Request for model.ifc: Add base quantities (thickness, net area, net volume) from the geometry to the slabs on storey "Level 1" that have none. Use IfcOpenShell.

First a look at what the model holds.

```python
import ifcopenshell
import ifcopenshell.util.element
import ifcopenshell.util.unit

model = ifcopenshell.open("model.ifc")
print(model.schema)
for unit_type in ("LENGTHUNIT", "AREAUNIT", "VOLUMEUNIT"):
    print(unit_type, ifcopenshell.util.unit.calculate_unit_scale(model, unit_type))
storey = next(s for s in model.by_type("IfcBuildingStorey") if s.Name == "Level 1")
slabs = [e for e in ifcopenshell.util.element.get_decomposition(storey) if e.is_a("IfcSlab")]
for e in sorted(slabs, key=lambda e: e.id()):
    print(e.id(), e.is_a(), e.Name, list(ifcopenshell.util.element.get_psets(e, qtos_only=True)), sep=" | ")
```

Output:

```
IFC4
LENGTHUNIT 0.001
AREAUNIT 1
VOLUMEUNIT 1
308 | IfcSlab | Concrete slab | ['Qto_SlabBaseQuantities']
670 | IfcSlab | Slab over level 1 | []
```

```python
import ifcopenshell
import ifcopenshell.api.pset
import ifcopenshell.geom
import ifcopenshell.util.element
import ifcopenshell.util.shape
import ifcopenshell.util.unit

model = ifcopenshell.open("model.ifc")
unit_scale = ifcopenshell.util.unit.calculate_unit_scale(model)
area_scale = ifcopenshell.util.unit.calculate_unit_scale(model, "AREAUNIT")
volume_scale = ifcopenshell.util.unit.calculate_unit_scale(model, "VOLUMEUNIT")
settings = ifcopenshell.geom.settings()

storey = next(s for s in model.by_type("IfcBuildingStorey") if s.Name == "Level 1")
slabs = [e for e in ifcopenshell.util.element.get_decomposition(storey) if e.is_a("IfcSlab")]

for e in sorted(slabs, key=lambda e: e.id()):
    if ifcopenshell.util.element.get_psets(e, qtos_only=True, should_inherit=False):
        continue
    # Geometry comes back in metres, in the element's own axes.
    shape = ifcopenshell.geom.create_shape(settings, e)
    values = {
        "Width": ifcopenshell.util.shape.get_z(shape.geometry) / unit_scale,
        "NetArea": ifcopenshell.util.shape.get_footprint_area(shape.geometry) / area_scale,
        "NetVolume": ifcopenshell.util.shape.get_volume(shape.geometry) / volume_scale,
    }
    qto = ifcopenshell.api.pset.add_qto(model, product=e, name="Qto_SlabBaseQuantities")
    ifcopenshell.api.pset.edit_qto(model, qto=qto, properties=values)
    print(e.id(), {k: round(v, 3) for k, v in values.items()})

model.write("model_v2.ifc")
```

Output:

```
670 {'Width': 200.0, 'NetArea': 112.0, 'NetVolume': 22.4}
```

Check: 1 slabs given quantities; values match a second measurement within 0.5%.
